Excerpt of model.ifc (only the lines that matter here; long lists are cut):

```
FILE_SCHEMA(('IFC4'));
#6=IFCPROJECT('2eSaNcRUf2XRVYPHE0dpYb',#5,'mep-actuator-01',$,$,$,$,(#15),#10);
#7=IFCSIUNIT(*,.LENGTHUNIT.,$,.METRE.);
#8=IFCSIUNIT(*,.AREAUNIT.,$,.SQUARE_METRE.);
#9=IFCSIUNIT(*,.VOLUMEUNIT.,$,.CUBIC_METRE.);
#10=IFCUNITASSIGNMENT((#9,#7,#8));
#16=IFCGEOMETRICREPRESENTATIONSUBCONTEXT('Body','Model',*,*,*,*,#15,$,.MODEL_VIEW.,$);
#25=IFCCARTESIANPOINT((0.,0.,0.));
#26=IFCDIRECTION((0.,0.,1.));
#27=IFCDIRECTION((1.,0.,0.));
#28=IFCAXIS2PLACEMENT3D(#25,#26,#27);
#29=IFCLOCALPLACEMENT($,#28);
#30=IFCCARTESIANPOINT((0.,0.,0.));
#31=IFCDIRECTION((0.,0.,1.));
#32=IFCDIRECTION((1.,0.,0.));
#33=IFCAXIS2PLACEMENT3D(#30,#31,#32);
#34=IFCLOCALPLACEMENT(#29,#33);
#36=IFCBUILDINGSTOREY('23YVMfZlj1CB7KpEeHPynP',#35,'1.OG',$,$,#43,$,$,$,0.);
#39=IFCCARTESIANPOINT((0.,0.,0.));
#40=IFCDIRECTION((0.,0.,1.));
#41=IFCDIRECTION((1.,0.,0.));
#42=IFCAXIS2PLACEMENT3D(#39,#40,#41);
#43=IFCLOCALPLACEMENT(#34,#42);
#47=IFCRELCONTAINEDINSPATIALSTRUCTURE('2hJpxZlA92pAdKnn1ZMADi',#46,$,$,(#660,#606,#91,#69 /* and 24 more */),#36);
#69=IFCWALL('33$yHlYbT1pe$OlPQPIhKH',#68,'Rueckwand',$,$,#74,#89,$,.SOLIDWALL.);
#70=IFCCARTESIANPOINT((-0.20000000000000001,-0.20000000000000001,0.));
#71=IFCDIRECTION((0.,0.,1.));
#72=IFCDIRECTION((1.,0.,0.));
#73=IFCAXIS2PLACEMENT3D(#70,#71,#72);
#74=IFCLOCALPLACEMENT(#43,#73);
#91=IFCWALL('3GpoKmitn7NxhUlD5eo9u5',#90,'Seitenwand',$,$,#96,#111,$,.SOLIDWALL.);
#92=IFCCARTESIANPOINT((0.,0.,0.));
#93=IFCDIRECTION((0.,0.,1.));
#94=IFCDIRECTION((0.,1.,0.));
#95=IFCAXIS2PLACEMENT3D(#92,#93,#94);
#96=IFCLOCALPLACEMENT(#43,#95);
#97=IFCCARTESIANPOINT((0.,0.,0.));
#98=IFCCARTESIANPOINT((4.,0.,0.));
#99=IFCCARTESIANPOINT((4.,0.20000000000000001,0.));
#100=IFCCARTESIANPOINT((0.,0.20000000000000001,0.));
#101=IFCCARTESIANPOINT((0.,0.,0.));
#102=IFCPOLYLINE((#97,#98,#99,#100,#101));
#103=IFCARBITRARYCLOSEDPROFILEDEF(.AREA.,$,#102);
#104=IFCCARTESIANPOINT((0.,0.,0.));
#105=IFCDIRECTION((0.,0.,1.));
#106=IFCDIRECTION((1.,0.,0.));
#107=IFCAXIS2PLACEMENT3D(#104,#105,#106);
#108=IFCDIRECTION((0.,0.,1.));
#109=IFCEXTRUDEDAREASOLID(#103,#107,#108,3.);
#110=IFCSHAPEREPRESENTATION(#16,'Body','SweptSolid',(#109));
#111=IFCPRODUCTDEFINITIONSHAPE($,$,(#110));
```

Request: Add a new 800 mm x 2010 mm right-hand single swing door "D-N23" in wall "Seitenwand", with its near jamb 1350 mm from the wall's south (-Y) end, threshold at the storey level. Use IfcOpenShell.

```python
import numpy as np
import ifcopenshell
import ifcopenshell.api.feature
import ifcopenshell.api.geometry
import ifcopenshell.api.root
import ifcopenshell.api.spatial
import ifcopenshell.geom
import ifcopenshell.util.element
import ifcopenshell.util.placement
import ifcopenshell.util.representation
import ifcopenshell.util.shape
import ifcopenshell.util.unit

model = ifcopenshell.open("model.ifc")
unit_scale = ifcopenshell.util.unit.calculate_unit_scale(model)
settings = ifcopenshell.geom.settings()


def volume(element):
    """Net volume in cubic metres, openings subtracted."""
    shape = ifcopenshell.geom.create_shape(settings, element)
    return ifcopenshell.util.shape.get_volume(shape.geometry)


wall = model.by_guid("3GpoKmitn7NxhUlD5eo9u5")
storey = ifcopenshell.util.element.get_container(wall, ifc_class="IfcBuildingStorey")
context = ifcopenshell.util.representation.get_context(model, "Model", "Body", "MODEL_VIEW")
before = volume(wall)

width, height, from_end, sill = 0.8, 2.01, 1.35, 0.0  # metres

# The wall runs along its own X axis, and the end named is its -X end.
wall_shape = ifcopenshell.geom.create_shape(settings, wall)
x, y, z = ifcopenshell.util.shape.get_vertices(wall_shape.geometry).T
start = x.min() + from_end
face, thickness = float(y.min()), float(y.max() - y.min())
wall_matrix = ifcopenshell.util.placement.get_local_placement(wall.ObjectPlacement)
level = ifcopenshell.util.placement.get_local_placement(storey.ObjectPlacement)[2, 3]


def in_wall(x, y):
    """Placement at x, y metres in the wall's axes, at sill height."""
    matrix = wall_matrix.copy()
    matrix[:, 3] = wall_matrix @ np.array([x / unit_scale, y / unit_scale, 0.0, 1.0])
    matrix[2, 3] = level + sill / unit_scale
    return matrix


# Opening: a box that overshoots both wall faces by 50 mm.
opening = ifcopenshell.api.root.create_entity(model, ifc_class="IfcOpeningElement", predefined_type="OPENING")
box = ifcopenshell.api.geometry.add_wall_representation(
    model, context=context, length=width, height=height, thickness=thickness + 0.1
)
ifcopenshell.api.geometry.assign_representation(model, product=opening, representation=box)
ifcopenshell.api.geometry.edit_object_placement(model, product=opening, matrix=in_wall(start, face - 0.05), is_si=False)
ifcopenshell.api.feature.add_feature(model, feature=opening, element=wall)

door = ifcopenshell.api.root.create_entity(model, ifc_class="IfcDoor", name="D-N23", predefined_type="DOOR")
door.OverallWidth, door.OverallHeight = width / unit_scale, height / unit_scale
door.OperationType = "SINGLE_SWING_RIGHT"
body = ifcopenshell.api.geometry.add_door_representation(
    model,
    context=context,
    overall_width=door.OverallWidth,
    overall_height=door.OverallHeight,
    operation_type="SINGLE_SWING_RIGHT",
    lining_properties={"LiningDepth": thickness / unit_scale, "ThresholdDepth": thickness / unit_scale},
)
ifcopenshell.api.geometry.assign_representation(model, product=door, representation=body)
ifcopenshell.api.spatial.assign_container(model, products=[door], relating_structure=storey)
ifcopenshell.api.feature.add_filling(model, opening=opening, element=door)

# The lining spans the wall, so the door starts at the wall face.
ifcopenshell.api.geometry.edit_object_placement(model, product=door, matrix=in_wall(start, face), is_si=False)

after = volume(wall)

print(f"wall volume {before:.3f} -> {after:.3f} m3")

model.write("model-out.ifc")
```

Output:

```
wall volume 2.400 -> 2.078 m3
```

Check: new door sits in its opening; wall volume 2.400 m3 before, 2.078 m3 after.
